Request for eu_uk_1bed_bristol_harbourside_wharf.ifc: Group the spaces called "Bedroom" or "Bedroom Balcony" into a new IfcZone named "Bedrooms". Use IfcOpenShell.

First a look at what the model holds.

```python
import ifcopenshell

model = ifcopenshell.open("eu_uk_1bed_bristol_harbourside_wharf.ifc")
print(model.schema)
seen = {}
for space in model.by_type("IfcSpace"):
    seen[space.LongName] = seen.get(space.LongName, 0) + 1
for name, count in sorted(seen.items(), key=str):
    print(count, "x", name)
print("zones:", [z.Name for z in model.by_type("IfcZone")][:20])
```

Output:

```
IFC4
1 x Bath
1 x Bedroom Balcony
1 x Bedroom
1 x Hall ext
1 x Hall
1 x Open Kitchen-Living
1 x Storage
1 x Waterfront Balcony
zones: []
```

```python
import ifcopenshell
import ifcopenshell.api.group
import ifcopenshell.api.root

model = ifcopenshell.open("eu_uk_1bed_bristol_harbourside_wharf.ifc")

names = {"Bedroom", "Bedroom Balcony"}
spaces = [s for s in model.by_type("IfcSpace") if s.LongName in names]

zone = ifcopenshell.api.root.create_entity(model, ifc_class="IfcZone", name="Bedrooms")
ifcopenshell.api.group.assign_group(model, products=spaces, group=zone)
print(len(spaces), "spaces in", zone.Name)

model.write("eu_uk_1bed_bristol_harbourside_wharf_v2.ifc")
```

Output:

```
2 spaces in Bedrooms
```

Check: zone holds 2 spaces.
